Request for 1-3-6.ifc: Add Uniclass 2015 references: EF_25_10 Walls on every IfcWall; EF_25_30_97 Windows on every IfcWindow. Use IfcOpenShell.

First a look at what the model holds.

```python
import ifcopenshell

model = ifcopenshell.open("1-3-6.ifc")
print(model.schema)
print("classifications:", [c.Name for c in model.by_type("IfcClassification")])
for ifc_class in ("IfcDoor", "IfcRoof", "IfcStair", "IfcWall", "IfcWindow"):
    print(ifc_class, len(model.by_type(ifc_class)))
```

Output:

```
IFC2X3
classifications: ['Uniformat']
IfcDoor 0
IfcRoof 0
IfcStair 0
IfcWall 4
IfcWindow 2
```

```python
import ifcopenshell
import ifcopenshell.api.classification

model = ifcopenshell.open("1-3-6.ifc")

# IFC2X3 requires Source and Edition and has no link from the project to the system.
system = model.create_entity("IfcClassification", Source="NBS", Edition="2015", Name="Uniclass 2015")

codes = {
    "IfcWall": ("EF_25_10", "Walls"),
    "IfcWindow": ("EF_25_30_97", "Windows"),
}
for ifc_class, (code, name) in codes.items():
    products = model.by_type(ifc_class)
    ifcopenshell.api.classification.add_reference(
        model, products=products, classification=system, identification=code, name=name
    )
    print(code, len(products))

model.write("1-3-6_updated.ifc")
```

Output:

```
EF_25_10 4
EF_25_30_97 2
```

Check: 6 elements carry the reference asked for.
